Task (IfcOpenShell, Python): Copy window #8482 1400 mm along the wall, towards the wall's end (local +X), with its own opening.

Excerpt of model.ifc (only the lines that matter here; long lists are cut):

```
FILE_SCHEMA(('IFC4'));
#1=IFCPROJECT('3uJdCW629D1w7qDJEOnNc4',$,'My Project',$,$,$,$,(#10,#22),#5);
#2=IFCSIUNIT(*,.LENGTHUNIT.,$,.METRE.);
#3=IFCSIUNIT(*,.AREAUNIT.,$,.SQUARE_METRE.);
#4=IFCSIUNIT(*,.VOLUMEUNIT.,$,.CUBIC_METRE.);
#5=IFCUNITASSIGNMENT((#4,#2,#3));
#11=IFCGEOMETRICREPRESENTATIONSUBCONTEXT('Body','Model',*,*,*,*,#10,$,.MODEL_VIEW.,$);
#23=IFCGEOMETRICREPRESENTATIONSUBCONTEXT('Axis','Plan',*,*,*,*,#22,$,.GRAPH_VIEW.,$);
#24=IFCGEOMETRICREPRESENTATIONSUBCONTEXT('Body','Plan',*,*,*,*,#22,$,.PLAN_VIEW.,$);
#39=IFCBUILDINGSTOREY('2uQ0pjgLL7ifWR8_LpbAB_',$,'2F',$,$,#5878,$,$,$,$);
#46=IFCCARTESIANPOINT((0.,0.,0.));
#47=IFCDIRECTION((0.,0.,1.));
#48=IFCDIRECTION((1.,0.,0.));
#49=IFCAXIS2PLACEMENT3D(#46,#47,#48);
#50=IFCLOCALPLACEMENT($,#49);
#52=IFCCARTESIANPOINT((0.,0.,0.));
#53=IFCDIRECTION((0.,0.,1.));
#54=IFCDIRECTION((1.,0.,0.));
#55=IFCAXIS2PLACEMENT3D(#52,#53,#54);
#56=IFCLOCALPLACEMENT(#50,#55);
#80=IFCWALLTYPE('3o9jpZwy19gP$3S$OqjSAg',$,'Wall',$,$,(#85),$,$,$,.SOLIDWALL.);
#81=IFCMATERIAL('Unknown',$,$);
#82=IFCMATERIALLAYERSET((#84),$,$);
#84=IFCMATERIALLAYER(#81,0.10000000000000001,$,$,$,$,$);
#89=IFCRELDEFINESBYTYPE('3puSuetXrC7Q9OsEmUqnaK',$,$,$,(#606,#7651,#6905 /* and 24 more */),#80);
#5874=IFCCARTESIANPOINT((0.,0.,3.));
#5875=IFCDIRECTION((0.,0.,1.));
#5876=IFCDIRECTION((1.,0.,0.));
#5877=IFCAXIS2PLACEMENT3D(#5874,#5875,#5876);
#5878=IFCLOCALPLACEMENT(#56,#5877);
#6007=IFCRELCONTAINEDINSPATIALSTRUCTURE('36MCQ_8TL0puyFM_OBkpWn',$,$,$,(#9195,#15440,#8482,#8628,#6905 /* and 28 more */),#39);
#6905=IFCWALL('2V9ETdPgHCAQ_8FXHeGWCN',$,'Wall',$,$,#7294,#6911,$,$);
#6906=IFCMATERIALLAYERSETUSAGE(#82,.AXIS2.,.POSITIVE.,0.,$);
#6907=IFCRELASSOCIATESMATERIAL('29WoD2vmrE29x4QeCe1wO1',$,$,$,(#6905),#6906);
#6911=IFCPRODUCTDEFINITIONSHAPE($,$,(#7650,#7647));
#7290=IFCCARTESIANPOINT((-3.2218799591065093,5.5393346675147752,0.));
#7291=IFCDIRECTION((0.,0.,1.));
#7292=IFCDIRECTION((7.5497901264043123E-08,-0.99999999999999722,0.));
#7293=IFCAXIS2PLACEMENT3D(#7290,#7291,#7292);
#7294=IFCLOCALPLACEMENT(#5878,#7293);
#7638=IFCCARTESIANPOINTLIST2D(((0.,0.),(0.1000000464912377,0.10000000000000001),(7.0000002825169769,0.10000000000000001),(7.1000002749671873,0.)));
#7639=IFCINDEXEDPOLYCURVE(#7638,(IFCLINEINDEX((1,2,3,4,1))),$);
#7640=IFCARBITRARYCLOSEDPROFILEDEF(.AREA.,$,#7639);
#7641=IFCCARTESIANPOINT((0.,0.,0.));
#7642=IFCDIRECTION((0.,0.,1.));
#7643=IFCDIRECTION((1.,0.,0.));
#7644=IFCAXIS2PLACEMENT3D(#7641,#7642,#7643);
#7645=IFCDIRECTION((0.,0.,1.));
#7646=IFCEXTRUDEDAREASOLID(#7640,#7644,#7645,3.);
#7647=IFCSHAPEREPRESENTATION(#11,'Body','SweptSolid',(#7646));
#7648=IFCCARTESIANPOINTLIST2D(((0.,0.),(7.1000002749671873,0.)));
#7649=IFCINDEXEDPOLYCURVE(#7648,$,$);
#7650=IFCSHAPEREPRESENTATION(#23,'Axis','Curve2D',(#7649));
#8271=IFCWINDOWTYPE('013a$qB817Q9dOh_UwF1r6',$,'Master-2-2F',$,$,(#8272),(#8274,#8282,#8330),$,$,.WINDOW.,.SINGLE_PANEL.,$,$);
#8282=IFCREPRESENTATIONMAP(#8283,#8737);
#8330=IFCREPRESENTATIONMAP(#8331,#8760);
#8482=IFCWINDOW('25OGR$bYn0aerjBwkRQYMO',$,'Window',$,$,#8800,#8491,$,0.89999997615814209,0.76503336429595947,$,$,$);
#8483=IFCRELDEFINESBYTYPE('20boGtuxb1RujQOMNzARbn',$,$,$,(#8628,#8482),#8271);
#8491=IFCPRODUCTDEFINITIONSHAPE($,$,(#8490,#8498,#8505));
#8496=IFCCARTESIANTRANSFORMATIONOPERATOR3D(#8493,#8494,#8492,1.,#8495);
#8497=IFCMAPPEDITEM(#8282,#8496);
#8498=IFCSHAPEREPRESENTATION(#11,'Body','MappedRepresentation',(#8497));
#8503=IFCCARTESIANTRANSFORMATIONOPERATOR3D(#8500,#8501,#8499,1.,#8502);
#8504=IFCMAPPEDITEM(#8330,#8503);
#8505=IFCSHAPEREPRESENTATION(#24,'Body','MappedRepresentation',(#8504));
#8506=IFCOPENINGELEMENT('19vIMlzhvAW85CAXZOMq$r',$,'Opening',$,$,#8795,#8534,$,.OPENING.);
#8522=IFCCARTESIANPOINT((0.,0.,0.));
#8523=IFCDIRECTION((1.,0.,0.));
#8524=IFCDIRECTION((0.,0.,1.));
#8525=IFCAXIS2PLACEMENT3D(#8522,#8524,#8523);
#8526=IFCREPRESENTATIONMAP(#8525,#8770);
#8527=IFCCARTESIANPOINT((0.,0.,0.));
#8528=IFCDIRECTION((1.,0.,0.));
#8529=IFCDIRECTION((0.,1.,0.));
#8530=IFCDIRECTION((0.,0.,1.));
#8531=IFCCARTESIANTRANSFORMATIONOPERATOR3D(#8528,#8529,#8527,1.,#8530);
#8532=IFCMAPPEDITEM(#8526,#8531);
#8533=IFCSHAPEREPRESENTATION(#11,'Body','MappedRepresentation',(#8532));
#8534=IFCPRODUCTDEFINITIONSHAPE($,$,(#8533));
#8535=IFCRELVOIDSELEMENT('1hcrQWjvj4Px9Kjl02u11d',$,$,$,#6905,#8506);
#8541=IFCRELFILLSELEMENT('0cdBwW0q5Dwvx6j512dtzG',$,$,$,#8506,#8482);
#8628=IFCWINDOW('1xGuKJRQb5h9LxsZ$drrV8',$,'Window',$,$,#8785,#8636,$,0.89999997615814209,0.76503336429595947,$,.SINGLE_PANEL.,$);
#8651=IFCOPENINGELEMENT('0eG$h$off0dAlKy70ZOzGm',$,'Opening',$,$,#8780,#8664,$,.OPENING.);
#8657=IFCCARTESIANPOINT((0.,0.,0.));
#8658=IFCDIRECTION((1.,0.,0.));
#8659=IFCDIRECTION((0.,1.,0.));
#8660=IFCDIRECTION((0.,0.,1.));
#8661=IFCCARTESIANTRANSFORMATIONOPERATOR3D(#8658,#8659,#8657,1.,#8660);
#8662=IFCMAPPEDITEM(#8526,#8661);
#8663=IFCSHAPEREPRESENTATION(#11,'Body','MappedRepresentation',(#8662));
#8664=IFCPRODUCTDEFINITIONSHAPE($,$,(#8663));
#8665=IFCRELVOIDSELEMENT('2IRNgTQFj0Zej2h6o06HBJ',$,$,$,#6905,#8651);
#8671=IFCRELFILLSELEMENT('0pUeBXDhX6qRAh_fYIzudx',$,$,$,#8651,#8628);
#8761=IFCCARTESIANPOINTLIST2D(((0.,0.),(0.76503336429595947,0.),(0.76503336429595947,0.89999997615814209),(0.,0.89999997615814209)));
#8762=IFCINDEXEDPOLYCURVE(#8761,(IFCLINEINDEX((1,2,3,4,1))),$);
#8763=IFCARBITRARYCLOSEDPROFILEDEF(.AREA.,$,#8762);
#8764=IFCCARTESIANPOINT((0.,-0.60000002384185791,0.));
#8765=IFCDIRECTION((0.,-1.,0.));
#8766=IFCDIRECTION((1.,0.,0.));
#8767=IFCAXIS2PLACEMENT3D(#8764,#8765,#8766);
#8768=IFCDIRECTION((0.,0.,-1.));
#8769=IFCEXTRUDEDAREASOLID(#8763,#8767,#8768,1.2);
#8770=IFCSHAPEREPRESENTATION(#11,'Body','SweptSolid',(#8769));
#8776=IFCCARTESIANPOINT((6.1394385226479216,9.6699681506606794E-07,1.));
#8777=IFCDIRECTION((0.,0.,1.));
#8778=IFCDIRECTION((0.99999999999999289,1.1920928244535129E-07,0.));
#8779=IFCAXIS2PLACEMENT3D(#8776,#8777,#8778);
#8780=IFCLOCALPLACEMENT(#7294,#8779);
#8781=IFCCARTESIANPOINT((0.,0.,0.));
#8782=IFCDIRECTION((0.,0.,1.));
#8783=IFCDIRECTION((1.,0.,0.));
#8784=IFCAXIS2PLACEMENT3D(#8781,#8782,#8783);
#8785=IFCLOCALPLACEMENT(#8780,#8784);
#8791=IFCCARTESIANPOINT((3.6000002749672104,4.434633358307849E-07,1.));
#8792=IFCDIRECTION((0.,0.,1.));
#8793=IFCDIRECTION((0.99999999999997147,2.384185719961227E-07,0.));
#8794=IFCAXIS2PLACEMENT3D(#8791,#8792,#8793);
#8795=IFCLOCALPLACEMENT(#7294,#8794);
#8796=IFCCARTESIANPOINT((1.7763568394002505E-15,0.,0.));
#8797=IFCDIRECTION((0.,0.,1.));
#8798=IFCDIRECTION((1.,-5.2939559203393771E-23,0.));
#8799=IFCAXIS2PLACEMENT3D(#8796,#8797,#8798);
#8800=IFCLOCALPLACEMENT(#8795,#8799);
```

```python
import ifcopenshell
import ifcopenshell.api.feature
import ifcopenshell.api.geometry
import ifcopenshell.api.root
import ifcopenshell.geom
import ifcopenshell.util.element
import ifcopenshell.util.placement
import ifcopenshell.util.shape

model = ifcopenshell.open("model.ifc")
settings = ifcopenshell.geom.settings()


def volume(element):
    """Net volume in cubic metres, openings subtracted."""
    shape = ifcopenshell.geom.create_shape(settings, element)
    return ifcopenshell.util.shape.get_volume(shape.geometry)


window = model.by_id(8482)
opening = window.FillsVoids[0].RelatingOpeningElement
wall = opening.VoidsElements[0].RelatingBuildingElement
before = volume(wall)
shift = ifcopenshell.util.placement.get_local_placement(wall.ObjectPlacement)[:3, 0] * 1.4

# copy_class copies the void relationship, type, container and properties, but no geometry.
new_opening = ifcopenshell.api.root.copy_class(model, product=opening)
new_opening.Representation = ifcopenshell.util.element.copy_deep(
    model, opening.Representation, exclude=["IfcGeometricRepresentationContext", "IfcRepresentationMap"]
)
new_window = ifcopenshell.api.root.copy_class(model, product=window)
new_window.Representation = ifcopenshell.util.element.copy_deep(
    model, window.Representation, exclude=["IfcGeometricRepresentationContext", "IfcRepresentationMap"]
)
ifcopenshell.api.feature.add_filling(model, opening=new_opening, element=new_window)

for old, new in ((opening, new_opening), (window, new_window)):
    matrix = ifcopenshell.util.placement.get_local_placement(old.ObjectPlacement)
    matrix[:3, 3] += shift
    ifcopenshell.api.geometry.edit_object_placement(model, product=new, matrix=matrix, is_si=False)

after = volume(wall)

print(f"wall volume {before:.3f} -> {after:.3f} m3")

model.write("model_rev.ifc")
```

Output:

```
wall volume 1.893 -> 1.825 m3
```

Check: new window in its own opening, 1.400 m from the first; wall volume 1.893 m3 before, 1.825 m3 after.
